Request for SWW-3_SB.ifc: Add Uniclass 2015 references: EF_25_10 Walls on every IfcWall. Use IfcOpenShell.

First a look at what the model holds.

```python
import ifcopenshell

model = ifcopenshell.open("SWW-3_SB.ifc")
print(model.schema)
print("classifications:", [c.Name for c in model.by_type("IfcClassification")])
for ifc_class in ("IfcDoor", "IfcRoof", "IfcStair", "IfcWall", "IfcWindow"):
    print(ifc_class, len(model.by_type(ifc_class)))
```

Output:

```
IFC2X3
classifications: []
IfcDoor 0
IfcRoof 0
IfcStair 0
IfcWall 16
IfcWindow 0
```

```python
import ifcopenshell
import ifcopenshell.api.classification

model = ifcopenshell.open("SWW-3_SB.ifc")

# IFC2X3 requires Source and Edition and has no link from the project to the system.
system = model.create_entity("IfcClassification", Source="NBS", Edition="2015", Name="Uniclass 2015")

codes = {
    "IfcWall": ("EF_25_10", "Walls"),
}
for ifc_class, (code, name) in codes.items():
    products = model.by_type(ifc_class)
    ifcopenshell.api.classification.add_reference(
        model, products=products, classification=system, identification=code, name=name
    )
    print(code, len(products))

model.write("SWW-3_SB_edited.ifc")
```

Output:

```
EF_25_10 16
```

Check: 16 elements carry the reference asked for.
